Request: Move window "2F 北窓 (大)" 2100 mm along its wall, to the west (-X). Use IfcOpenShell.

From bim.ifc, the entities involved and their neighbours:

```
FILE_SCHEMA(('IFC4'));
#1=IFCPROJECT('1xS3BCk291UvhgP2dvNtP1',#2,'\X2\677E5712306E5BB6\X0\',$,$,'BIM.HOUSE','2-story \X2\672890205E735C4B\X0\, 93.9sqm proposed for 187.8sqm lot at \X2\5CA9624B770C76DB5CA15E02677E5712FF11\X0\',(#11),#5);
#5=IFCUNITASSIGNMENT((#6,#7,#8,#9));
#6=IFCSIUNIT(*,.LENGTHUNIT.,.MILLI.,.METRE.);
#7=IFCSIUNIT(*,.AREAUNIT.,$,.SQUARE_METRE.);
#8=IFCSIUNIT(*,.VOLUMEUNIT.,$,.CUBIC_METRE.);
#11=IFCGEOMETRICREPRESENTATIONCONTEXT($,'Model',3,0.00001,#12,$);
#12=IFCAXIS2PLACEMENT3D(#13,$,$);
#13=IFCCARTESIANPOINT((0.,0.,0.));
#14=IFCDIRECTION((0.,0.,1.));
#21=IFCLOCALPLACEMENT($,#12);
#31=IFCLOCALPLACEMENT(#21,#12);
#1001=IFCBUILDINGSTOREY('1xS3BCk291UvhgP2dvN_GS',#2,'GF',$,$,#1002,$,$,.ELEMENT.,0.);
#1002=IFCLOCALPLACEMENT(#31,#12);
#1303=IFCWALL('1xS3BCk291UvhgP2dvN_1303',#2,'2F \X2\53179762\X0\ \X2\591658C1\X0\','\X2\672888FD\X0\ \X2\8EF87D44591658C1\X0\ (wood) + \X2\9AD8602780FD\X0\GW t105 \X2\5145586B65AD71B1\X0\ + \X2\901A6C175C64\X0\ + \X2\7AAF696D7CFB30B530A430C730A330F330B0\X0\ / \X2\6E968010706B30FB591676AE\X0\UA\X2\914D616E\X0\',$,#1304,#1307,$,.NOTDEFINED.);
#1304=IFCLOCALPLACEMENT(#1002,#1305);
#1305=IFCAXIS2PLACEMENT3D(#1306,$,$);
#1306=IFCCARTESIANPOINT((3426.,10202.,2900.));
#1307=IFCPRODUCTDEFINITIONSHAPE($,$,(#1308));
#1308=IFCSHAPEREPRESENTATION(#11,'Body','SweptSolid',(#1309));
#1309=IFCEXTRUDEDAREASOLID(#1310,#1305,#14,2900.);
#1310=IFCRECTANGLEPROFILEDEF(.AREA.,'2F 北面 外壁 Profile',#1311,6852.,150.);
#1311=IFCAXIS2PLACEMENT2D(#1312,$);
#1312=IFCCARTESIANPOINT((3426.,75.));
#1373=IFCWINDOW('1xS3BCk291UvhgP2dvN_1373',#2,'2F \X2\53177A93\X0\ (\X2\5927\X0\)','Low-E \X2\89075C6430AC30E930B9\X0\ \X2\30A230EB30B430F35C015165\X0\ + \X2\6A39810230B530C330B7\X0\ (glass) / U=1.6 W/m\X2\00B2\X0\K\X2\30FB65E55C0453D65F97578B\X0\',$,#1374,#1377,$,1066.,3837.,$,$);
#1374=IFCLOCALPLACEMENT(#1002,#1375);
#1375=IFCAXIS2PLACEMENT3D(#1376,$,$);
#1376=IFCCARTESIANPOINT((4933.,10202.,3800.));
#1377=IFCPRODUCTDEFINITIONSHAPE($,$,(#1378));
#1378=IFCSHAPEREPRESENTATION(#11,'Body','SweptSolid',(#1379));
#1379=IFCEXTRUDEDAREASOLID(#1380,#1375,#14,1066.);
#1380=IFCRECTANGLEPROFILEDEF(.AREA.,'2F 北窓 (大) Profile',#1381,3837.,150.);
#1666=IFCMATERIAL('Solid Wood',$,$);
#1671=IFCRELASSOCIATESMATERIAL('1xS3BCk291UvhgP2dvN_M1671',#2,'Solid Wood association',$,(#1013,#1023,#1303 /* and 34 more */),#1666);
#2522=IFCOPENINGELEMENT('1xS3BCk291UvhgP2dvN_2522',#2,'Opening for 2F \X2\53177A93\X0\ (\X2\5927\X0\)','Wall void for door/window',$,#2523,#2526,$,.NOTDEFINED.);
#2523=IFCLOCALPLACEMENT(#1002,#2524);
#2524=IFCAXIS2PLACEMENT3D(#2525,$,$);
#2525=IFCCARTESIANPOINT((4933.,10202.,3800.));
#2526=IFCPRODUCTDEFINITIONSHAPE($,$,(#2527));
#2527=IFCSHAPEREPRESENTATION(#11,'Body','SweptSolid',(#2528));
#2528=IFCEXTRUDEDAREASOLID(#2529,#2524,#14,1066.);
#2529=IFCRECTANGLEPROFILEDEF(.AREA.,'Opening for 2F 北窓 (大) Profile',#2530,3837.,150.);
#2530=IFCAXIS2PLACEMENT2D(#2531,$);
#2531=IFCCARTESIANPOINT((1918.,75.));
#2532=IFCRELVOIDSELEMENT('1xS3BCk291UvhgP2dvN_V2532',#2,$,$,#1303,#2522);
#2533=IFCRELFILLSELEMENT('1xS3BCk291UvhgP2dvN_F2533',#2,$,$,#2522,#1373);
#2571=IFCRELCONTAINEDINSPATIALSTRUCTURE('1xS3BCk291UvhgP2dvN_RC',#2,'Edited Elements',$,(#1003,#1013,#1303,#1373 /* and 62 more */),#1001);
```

```python
import ifcopenshell
import ifcopenshell.api.geometry
import ifcopenshell.util.placement
import ifcopenshell.util.unit

model = ifcopenshell.open("bim.ifc")
unit_scale = ifcopenshell.util.unit.calculate_unit_scale(model)

window = model.by_id(1373)
opening = window.FillsVoids[0].RelatingOpeningElement
wall = opening.VoidsElements[0].RelatingBuildingElement

wall_matrix = ifcopenshell.util.placement.get_local_placement(wall.ObjectPlacement)
shift = wall_matrix[:3, 0] * -2.1 / unit_scale
before = ifcopenshell.util.placement.get_local_placement(window.ObjectPlacement)[:3, 3].copy()

# The window is not placed relative to its opening, so move both.
for product in (opening, window):
    matrix = ifcopenshell.util.placement.get_local_placement(product.ObjectPlacement)
    matrix[:3, 3] += shift
    ifcopenshell.api.geometry.edit_object_placement(model, product=product, matrix=matrix, is_si=False)

after = ifcopenshell.util.placement.get_local_placement(window.ObjectPlacement)[:3, 3]
print("window moved by", (after - before).round(3) + 0.0)

model.write("bim_v2.ifc")
```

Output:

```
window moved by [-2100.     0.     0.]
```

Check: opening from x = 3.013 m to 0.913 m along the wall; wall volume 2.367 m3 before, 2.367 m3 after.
